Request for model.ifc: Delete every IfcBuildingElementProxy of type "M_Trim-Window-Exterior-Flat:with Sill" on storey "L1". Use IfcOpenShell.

First a look at what the model holds.

```python
import ifcopenshell
import ifcopenshell.util.element

model = ifcopenshell.open("model.ifc")
print(model.schema)
storey = next(s for s in model.by_type("IfcBuildingStorey") if s.Name == "L1")
proxies = [e for e in ifcopenshell.util.element.get_decomposition(storey) if e.is_a("IfcBuildingElementProxy")]
seen = {}
for e in proxies:
    element_type = ifcopenshell.util.element.get_type(e)
    name = element_type.Name if element_type not in (None, e) else None
    seen[name] = seen.get(name, 0) + 1
for name, count in sorted(seen.items(), key=str):
    print(count, "x", name)
```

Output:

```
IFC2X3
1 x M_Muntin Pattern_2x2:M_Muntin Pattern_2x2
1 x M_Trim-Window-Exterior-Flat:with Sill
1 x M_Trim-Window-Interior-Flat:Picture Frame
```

```python
import ifcopenshell
import ifcopenshell.api.root
import ifcopenshell.util.element

model = ifcopenshell.open("model.ifc")

storey = next(s for s in model.by_type("IfcBuildingStorey") if s.Name == "L1")
proxies = [e for e in ifcopenshell.util.element.get_decomposition(storey) if e.is_a("IfcBuildingElementProxy")]
targets = [e for e in proxies if (t := ifcopenshell.util.element.get_type(e)) not in (None, e) and t.Name == "M_Trim-Window-Exterior-Flat:with Sill"]

for e in targets:
    ifcopenshell.api.root.remove_product(model, product=e)
print(len(targets), "removed")

model.write("model_edited.ifc")
```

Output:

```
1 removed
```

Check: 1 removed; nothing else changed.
